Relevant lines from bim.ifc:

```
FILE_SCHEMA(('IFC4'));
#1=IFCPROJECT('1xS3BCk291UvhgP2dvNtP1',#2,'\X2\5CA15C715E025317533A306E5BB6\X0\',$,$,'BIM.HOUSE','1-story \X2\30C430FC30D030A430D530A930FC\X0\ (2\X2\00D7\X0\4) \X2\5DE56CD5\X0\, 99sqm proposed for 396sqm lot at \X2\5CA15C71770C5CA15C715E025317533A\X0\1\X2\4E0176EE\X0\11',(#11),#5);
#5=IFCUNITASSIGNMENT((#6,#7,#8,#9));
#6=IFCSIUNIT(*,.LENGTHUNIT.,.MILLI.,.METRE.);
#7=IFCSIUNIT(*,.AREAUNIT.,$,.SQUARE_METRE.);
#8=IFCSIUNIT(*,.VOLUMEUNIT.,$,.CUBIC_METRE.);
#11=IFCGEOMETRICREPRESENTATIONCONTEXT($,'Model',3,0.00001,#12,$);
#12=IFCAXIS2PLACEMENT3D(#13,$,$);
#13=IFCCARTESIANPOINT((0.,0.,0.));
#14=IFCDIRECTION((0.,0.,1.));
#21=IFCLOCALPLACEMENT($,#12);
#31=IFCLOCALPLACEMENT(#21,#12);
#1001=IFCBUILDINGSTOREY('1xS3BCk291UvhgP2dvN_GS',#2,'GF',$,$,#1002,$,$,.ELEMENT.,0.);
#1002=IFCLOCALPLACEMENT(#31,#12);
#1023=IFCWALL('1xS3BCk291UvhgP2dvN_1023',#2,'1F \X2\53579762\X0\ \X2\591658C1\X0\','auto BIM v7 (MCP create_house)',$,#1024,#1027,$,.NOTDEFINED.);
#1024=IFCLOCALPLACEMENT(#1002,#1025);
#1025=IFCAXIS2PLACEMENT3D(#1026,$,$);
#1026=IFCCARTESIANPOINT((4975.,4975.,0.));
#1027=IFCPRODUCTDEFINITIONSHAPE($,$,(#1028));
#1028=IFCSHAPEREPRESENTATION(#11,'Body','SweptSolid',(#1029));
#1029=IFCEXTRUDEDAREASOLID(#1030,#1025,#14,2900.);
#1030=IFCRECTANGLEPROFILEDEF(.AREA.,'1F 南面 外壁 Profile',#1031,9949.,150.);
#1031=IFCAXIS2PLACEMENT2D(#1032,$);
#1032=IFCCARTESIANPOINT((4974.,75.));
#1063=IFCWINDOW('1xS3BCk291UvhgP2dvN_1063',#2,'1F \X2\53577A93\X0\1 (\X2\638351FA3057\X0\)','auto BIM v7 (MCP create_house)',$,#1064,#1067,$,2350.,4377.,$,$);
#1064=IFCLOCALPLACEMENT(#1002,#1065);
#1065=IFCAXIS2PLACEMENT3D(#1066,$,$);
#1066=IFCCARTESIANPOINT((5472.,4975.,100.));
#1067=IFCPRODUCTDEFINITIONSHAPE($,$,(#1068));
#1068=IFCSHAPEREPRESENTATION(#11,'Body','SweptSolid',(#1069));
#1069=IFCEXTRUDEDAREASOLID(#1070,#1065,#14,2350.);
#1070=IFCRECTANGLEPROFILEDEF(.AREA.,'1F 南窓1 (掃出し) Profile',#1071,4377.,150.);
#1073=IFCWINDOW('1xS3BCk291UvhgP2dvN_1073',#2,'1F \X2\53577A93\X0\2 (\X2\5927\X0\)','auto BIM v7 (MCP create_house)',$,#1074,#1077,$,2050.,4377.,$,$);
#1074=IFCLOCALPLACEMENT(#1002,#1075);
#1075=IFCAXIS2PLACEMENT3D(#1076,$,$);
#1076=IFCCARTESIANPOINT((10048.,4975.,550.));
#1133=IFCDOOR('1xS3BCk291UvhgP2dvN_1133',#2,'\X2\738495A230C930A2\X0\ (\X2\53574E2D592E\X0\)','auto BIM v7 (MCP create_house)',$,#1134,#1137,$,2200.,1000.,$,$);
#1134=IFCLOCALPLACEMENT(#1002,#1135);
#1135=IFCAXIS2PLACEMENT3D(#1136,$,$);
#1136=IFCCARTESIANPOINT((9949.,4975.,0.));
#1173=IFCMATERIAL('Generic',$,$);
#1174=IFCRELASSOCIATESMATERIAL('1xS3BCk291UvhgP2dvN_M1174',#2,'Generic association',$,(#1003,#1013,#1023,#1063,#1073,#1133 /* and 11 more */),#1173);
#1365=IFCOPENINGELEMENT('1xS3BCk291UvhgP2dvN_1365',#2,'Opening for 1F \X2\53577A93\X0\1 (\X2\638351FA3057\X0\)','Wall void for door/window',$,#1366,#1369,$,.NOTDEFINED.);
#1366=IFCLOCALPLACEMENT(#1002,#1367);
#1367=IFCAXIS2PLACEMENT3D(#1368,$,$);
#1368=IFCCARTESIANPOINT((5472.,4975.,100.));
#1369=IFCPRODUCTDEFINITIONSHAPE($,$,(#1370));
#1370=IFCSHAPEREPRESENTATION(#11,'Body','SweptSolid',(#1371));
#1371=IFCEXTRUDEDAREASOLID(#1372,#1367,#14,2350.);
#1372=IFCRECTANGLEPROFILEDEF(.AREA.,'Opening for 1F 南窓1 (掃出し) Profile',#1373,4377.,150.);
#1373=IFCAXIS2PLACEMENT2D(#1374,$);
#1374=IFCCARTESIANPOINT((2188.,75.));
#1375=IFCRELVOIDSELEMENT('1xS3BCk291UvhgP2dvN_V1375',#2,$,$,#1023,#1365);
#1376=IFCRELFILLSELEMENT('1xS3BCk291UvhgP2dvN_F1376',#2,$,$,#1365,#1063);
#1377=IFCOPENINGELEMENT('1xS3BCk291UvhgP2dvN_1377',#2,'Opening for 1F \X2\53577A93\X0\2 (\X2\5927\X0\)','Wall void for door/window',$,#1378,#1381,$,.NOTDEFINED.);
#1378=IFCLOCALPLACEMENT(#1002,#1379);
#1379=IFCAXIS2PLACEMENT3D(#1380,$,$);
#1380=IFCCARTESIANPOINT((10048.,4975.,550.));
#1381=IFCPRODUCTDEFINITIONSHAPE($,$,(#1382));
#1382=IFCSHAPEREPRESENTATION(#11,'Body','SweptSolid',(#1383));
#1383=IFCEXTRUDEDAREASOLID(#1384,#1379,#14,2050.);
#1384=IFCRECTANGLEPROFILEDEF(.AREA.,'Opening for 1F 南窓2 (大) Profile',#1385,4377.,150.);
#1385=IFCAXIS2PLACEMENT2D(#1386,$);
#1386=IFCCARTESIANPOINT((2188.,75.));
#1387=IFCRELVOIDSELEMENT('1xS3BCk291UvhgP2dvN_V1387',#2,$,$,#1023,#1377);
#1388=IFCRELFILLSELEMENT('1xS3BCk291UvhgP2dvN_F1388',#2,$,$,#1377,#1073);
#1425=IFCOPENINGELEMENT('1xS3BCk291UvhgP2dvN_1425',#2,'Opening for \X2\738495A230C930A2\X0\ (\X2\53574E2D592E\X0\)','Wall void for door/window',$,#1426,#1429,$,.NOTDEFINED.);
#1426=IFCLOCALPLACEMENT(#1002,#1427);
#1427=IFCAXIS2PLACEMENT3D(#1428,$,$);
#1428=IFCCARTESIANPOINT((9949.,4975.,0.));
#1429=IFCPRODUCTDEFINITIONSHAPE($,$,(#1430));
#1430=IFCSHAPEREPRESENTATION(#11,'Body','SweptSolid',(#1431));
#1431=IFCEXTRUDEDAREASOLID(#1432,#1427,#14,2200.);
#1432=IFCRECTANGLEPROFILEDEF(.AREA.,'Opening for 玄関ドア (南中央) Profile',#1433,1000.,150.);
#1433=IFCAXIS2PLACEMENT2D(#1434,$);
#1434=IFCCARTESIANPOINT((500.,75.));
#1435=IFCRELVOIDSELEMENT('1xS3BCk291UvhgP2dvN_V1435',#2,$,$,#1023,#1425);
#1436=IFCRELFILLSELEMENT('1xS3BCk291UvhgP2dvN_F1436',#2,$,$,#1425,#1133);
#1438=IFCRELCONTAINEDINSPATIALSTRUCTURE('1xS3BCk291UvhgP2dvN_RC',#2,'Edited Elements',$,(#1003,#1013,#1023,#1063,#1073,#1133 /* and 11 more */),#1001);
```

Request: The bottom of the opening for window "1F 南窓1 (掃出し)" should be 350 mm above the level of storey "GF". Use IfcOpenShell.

```python
import numpy as np
import ifcopenshell
import ifcopenshell.api.geometry
import ifcopenshell.geom
import ifcopenshell.util.element
import ifcopenshell.util.placement
import ifcopenshell.util.shape
import ifcopenshell.util.unit

model = ifcopenshell.open("bim.ifc")
unit_scale = ifcopenshell.util.unit.calculate_unit_scale(model)

window = model.by_id(1063)
opening = window.FillsVoids[0].RelatingOpeningElement
storey = ifcopenshell.util.element.get_container(window, ifc_class="IfcBuildingStorey")
level = ifcopenshell.util.placement.get_local_placement(storey.ObjectPlacement)[2, 3]

# The opening's origin need not be at the sill, so measure its lowest point.
shape = ifcopenshell.geom.create_shape(ifcopenshell.geom.settings(), opening)
bottom = ifcopenshell.util.shape.get_shape_bottom_elevation(shape, shape.geometry) / unit_scale
dz = level + 350.0 - bottom

shift = np.array([0.0, 0.0, dz])
# The window is not placed relative to its opening, so move both.
for product in (opening, window):
    matrix = ifcopenshell.util.placement.get_local_placement(product.ObjectPlacement)
    matrix[:3, 3] += shift
    ifcopenshell.api.geometry.edit_object_placement(model, product=product, matrix=matrix, is_si=False)

print(f"moved by {dz * unit_scale:+.3f} m")

model.write("bim_rev.ifc")
```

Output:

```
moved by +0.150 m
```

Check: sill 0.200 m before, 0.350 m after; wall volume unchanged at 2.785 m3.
